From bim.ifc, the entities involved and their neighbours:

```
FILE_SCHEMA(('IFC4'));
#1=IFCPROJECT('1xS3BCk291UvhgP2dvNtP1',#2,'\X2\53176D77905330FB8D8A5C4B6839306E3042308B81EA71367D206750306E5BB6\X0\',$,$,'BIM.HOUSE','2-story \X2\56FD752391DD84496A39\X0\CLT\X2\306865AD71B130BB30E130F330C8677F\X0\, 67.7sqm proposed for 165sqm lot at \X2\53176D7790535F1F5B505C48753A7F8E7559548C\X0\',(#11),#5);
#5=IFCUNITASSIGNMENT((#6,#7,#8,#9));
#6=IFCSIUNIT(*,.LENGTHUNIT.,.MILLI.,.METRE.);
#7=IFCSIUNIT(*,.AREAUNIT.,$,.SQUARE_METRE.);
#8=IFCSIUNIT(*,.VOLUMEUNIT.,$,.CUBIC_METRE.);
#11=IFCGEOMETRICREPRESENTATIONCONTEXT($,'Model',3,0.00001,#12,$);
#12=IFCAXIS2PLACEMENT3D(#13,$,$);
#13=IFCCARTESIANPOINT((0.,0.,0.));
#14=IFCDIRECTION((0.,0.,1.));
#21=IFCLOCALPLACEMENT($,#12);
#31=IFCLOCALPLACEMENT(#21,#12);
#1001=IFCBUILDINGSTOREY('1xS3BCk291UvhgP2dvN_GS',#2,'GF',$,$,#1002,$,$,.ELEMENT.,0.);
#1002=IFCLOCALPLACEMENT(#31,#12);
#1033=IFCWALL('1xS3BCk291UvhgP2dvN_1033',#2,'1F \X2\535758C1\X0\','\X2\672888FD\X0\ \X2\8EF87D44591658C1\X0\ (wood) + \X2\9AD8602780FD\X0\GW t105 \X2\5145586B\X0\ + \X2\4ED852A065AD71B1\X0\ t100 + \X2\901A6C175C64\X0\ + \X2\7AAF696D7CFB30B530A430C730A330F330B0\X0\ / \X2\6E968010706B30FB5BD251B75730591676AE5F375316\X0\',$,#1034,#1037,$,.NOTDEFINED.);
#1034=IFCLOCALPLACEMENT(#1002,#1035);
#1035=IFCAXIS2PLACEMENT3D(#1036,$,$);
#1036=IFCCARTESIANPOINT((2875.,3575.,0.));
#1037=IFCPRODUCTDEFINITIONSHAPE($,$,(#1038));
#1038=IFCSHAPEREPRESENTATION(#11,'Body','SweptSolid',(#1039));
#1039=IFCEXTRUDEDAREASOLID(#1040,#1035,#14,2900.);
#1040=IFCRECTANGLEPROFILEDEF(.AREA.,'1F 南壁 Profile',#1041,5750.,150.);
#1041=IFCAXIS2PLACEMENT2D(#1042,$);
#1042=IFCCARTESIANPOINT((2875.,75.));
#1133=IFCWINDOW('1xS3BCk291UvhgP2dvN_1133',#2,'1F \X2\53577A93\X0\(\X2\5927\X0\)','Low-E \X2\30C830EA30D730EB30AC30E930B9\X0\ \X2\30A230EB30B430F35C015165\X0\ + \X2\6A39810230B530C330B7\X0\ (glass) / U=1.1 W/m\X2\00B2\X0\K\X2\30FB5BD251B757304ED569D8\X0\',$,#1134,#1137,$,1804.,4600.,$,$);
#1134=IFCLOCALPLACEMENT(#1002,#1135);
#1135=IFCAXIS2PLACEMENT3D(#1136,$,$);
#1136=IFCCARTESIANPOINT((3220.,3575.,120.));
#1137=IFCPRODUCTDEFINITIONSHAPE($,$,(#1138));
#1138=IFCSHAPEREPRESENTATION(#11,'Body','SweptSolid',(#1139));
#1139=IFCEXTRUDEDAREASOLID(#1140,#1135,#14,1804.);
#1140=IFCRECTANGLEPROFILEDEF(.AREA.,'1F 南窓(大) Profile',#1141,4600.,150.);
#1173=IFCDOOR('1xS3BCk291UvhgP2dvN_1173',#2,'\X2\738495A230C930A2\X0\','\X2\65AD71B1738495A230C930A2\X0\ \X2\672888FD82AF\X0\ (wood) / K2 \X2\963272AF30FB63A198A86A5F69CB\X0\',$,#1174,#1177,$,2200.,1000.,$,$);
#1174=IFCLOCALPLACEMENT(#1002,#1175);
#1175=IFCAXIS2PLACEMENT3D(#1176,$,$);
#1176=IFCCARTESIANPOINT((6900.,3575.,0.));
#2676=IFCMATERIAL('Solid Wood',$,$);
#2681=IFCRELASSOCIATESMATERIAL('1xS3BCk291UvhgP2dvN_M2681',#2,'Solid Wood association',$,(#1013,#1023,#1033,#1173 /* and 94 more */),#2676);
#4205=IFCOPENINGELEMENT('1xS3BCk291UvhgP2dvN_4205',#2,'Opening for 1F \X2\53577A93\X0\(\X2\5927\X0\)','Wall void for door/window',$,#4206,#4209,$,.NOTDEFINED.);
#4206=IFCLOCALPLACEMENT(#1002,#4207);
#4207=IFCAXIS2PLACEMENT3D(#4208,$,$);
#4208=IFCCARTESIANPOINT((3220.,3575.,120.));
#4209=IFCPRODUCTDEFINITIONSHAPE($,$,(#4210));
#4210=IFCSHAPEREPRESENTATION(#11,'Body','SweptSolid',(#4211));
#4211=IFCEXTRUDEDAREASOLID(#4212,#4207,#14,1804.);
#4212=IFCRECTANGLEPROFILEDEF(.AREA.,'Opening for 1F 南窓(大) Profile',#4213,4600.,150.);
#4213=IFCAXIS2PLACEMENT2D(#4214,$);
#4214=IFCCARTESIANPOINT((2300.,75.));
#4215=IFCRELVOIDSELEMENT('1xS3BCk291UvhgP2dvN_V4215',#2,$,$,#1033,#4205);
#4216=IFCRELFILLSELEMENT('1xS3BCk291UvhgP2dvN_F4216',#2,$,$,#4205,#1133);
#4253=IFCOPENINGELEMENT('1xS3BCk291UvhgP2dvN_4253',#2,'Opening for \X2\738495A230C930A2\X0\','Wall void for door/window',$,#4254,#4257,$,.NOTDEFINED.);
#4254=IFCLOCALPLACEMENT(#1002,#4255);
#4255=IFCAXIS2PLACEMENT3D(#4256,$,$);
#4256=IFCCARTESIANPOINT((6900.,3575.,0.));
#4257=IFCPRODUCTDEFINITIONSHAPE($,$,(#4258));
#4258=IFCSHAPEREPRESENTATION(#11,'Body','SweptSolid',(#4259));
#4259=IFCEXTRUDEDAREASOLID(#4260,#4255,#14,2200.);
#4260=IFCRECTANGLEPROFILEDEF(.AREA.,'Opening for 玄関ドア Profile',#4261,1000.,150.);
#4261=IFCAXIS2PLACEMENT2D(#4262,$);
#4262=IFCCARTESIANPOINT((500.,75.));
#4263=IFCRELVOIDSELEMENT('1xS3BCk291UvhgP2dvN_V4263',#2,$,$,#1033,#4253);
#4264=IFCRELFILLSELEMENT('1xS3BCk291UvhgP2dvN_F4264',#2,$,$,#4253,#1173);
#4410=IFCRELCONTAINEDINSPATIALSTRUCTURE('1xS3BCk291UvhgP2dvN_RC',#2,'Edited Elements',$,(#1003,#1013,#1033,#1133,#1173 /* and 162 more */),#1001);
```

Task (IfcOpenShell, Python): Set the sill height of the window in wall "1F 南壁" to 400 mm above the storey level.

```python
import numpy as np
import ifcopenshell
import ifcopenshell.api.geometry
import ifcopenshell.geom
import ifcopenshell.util.element
import ifcopenshell.util.placement
import ifcopenshell.util.shape
import ifcopenshell.util.unit

model = ifcopenshell.open("bim.ifc")
unit_scale = ifcopenshell.util.unit.calculate_unit_scale(model)

window = model.by_id(1133)
opening = window.FillsVoids[0].RelatingOpeningElement
storey = ifcopenshell.util.element.get_container(window, ifc_class="IfcBuildingStorey")
level = ifcopenshell.util.placement.get_local_placement(storey.ObjectPlacement)[2, 3]

# The opening's origin need not be at the sill, so measure its lowest point.
shape = ifcopenshell.geom.create_shape(ifcopenshell.geom.settings(), opening)
bottom = ifcopenshell.util.shape.get_shape_bottom_elevation(shape, shape.geometry) / unit_scale
dz = level + 400.0 - bottom

shift = np.array([0.0, 0.0, dz])
# The window is not placed relative to its opening, so move both.
for product in (opening, window):
    matrix = ifcopenshell.util.placement.get_local_placement(product.ObjectPlacement)
    matrix[:3, 3] += shift
    ifcopenshell.api.geometry.edit_object_placement(model, product=product, matrix=matrix, is_si=False)

print(f"moved by {dz * unit_scale:+.3f} m")

model.write("bim-out.ifc")
```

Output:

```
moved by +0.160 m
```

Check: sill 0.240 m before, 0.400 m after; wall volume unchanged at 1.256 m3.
